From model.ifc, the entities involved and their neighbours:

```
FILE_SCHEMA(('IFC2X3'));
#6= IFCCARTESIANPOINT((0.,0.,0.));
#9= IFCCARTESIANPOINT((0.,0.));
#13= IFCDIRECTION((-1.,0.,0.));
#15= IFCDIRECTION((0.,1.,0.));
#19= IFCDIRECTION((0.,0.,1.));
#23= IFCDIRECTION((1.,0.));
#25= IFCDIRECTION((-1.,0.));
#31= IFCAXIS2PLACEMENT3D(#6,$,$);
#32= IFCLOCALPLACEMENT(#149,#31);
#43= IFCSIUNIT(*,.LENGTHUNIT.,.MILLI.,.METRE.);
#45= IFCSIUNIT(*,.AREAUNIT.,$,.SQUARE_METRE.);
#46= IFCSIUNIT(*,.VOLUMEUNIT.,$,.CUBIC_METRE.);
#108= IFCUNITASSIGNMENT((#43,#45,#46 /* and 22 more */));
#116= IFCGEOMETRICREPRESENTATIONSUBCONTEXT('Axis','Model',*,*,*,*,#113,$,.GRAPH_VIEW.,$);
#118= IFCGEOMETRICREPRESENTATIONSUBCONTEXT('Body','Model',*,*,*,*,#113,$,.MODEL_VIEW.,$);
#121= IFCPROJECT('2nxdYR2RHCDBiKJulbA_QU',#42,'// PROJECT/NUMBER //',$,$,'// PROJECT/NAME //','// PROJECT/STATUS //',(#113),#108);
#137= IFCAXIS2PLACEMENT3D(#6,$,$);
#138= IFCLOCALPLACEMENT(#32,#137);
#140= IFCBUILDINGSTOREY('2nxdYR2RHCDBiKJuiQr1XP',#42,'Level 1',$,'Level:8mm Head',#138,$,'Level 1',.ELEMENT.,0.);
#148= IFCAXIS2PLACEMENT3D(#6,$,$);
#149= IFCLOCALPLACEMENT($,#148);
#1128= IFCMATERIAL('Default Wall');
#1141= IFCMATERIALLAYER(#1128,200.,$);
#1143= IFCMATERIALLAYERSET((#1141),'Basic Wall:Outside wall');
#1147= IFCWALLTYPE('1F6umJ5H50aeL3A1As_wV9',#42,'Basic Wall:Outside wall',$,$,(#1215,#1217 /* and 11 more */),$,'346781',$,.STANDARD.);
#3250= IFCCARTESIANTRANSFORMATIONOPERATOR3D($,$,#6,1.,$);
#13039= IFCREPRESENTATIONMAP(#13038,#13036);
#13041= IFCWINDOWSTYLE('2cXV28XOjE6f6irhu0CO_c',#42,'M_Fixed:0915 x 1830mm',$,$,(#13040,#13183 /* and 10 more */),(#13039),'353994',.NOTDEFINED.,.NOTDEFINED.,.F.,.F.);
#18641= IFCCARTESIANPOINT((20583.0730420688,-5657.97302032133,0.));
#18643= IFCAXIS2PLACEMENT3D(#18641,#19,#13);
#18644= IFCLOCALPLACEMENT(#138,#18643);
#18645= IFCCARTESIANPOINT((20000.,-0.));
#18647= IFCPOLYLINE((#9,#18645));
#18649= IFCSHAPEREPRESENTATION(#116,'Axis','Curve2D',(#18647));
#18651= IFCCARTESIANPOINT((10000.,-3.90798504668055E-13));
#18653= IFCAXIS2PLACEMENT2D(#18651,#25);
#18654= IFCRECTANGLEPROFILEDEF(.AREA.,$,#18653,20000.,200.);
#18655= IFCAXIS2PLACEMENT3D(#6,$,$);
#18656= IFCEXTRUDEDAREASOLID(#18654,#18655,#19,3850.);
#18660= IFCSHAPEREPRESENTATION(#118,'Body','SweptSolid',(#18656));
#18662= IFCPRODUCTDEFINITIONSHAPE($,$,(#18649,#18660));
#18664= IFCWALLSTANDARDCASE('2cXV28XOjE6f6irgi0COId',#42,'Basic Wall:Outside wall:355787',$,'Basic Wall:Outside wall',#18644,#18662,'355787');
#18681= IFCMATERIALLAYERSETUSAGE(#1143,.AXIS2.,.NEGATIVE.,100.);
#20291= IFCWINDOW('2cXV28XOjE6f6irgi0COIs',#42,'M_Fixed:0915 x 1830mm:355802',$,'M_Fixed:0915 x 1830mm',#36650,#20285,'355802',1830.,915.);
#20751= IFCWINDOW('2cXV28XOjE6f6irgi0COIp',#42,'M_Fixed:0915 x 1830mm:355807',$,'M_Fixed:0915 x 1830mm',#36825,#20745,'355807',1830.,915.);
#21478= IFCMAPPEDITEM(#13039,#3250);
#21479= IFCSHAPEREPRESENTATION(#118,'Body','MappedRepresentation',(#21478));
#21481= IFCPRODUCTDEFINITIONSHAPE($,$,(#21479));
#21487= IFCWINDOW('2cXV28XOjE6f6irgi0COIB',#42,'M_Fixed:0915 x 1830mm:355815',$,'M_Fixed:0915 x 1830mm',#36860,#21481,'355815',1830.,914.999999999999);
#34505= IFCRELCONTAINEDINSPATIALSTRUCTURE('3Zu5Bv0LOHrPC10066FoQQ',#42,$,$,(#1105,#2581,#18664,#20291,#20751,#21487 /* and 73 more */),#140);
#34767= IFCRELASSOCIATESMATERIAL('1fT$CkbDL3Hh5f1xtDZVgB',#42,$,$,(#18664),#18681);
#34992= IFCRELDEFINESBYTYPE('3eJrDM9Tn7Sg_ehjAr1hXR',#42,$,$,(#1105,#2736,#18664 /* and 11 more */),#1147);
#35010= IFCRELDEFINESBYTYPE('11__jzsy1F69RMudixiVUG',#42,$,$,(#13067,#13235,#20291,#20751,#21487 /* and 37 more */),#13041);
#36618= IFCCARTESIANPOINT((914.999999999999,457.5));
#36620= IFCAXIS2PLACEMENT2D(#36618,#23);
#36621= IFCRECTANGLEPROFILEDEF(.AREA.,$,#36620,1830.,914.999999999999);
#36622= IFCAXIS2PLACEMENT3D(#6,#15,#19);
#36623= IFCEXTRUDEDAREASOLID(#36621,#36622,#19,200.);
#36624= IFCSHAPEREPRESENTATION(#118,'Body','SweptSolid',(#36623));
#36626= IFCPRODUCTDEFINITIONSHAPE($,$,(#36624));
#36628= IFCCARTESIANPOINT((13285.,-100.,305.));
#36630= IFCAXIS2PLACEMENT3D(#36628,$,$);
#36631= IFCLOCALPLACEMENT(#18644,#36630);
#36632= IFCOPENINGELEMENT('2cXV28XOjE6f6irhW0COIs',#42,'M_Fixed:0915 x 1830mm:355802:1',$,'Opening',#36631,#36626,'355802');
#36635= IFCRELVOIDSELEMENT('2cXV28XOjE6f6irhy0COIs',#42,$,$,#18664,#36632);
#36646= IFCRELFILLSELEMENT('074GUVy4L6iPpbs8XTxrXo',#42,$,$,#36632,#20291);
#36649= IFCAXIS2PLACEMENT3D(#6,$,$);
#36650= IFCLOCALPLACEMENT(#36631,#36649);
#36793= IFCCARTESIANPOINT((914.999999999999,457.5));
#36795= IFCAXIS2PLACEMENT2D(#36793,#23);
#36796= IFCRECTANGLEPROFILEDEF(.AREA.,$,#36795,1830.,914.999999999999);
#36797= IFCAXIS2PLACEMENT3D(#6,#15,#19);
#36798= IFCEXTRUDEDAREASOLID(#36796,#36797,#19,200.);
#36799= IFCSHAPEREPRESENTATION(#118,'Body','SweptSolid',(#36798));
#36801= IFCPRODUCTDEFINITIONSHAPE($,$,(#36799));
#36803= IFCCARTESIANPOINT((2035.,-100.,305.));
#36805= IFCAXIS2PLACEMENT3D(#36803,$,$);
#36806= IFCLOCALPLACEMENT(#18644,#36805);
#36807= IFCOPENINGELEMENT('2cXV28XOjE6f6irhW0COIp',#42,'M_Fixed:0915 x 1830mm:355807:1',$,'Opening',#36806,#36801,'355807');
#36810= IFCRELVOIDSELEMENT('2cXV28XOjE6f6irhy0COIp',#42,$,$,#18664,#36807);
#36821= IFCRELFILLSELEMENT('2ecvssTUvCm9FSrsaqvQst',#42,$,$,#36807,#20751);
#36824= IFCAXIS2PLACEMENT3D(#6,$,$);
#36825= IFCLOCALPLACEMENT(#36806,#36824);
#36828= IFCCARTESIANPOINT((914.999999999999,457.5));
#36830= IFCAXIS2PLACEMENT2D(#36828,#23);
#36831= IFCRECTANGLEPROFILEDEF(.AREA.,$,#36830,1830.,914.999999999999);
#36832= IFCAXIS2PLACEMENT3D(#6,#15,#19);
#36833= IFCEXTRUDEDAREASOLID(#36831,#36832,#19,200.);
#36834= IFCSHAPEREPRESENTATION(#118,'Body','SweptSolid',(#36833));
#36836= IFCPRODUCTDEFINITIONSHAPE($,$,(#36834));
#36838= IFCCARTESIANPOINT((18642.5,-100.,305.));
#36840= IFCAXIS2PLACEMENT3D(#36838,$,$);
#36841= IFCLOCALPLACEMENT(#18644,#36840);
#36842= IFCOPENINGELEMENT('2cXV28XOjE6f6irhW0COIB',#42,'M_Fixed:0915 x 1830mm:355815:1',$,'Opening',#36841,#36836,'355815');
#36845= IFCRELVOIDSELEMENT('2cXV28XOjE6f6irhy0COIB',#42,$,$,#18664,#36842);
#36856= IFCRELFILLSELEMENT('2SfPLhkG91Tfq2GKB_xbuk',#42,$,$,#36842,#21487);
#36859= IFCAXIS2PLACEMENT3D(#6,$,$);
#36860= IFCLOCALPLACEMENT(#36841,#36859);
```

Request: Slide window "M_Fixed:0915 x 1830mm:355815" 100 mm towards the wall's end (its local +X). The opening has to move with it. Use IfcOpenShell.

```python
import ifcopenshell
import ifcopenshell.api.geometry
import ifcopenshell.util.placement

model = ifcopenshell.open("model.ifc")

window = model.by_guid("2cXV28XOjE6f6irgi0COIB")
opening = window.FillsVoids[0].RelatingOpeningElement
wall = opening.VoidsElements[0].RelatingBuildingElement

wall_matrix = ifcopenshell.util.placement.get_local_placement(wall.ObjectPlacement)
shift = wall_matrix[:3, 0] * 100.0
before = ifcopenshell.util.placement.get_local_placement(window.ObjectPlacement)[:3, 3].copy()

# The window is placed relative to its opening, so it follows when the opening moves.
matrix = ifcopenshell.util.placement.get_local_placement(opening.ObjectPlacement)
matrix[:3, 3] += shift
ifcopenshell.api.geometry.edit_object_placement(
    model, product=opening, matrix=matrix, is_si=False, should_transform_children=True
)

after = ifcopenshell.util.placement.get_local_placement(window.ObjectPlacement)[:3, 3]
print("window moved by", (after - before).round(3) + 0.0)

model.write("model_updated.ifc")
```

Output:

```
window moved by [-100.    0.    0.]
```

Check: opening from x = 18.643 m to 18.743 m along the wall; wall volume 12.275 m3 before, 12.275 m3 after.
